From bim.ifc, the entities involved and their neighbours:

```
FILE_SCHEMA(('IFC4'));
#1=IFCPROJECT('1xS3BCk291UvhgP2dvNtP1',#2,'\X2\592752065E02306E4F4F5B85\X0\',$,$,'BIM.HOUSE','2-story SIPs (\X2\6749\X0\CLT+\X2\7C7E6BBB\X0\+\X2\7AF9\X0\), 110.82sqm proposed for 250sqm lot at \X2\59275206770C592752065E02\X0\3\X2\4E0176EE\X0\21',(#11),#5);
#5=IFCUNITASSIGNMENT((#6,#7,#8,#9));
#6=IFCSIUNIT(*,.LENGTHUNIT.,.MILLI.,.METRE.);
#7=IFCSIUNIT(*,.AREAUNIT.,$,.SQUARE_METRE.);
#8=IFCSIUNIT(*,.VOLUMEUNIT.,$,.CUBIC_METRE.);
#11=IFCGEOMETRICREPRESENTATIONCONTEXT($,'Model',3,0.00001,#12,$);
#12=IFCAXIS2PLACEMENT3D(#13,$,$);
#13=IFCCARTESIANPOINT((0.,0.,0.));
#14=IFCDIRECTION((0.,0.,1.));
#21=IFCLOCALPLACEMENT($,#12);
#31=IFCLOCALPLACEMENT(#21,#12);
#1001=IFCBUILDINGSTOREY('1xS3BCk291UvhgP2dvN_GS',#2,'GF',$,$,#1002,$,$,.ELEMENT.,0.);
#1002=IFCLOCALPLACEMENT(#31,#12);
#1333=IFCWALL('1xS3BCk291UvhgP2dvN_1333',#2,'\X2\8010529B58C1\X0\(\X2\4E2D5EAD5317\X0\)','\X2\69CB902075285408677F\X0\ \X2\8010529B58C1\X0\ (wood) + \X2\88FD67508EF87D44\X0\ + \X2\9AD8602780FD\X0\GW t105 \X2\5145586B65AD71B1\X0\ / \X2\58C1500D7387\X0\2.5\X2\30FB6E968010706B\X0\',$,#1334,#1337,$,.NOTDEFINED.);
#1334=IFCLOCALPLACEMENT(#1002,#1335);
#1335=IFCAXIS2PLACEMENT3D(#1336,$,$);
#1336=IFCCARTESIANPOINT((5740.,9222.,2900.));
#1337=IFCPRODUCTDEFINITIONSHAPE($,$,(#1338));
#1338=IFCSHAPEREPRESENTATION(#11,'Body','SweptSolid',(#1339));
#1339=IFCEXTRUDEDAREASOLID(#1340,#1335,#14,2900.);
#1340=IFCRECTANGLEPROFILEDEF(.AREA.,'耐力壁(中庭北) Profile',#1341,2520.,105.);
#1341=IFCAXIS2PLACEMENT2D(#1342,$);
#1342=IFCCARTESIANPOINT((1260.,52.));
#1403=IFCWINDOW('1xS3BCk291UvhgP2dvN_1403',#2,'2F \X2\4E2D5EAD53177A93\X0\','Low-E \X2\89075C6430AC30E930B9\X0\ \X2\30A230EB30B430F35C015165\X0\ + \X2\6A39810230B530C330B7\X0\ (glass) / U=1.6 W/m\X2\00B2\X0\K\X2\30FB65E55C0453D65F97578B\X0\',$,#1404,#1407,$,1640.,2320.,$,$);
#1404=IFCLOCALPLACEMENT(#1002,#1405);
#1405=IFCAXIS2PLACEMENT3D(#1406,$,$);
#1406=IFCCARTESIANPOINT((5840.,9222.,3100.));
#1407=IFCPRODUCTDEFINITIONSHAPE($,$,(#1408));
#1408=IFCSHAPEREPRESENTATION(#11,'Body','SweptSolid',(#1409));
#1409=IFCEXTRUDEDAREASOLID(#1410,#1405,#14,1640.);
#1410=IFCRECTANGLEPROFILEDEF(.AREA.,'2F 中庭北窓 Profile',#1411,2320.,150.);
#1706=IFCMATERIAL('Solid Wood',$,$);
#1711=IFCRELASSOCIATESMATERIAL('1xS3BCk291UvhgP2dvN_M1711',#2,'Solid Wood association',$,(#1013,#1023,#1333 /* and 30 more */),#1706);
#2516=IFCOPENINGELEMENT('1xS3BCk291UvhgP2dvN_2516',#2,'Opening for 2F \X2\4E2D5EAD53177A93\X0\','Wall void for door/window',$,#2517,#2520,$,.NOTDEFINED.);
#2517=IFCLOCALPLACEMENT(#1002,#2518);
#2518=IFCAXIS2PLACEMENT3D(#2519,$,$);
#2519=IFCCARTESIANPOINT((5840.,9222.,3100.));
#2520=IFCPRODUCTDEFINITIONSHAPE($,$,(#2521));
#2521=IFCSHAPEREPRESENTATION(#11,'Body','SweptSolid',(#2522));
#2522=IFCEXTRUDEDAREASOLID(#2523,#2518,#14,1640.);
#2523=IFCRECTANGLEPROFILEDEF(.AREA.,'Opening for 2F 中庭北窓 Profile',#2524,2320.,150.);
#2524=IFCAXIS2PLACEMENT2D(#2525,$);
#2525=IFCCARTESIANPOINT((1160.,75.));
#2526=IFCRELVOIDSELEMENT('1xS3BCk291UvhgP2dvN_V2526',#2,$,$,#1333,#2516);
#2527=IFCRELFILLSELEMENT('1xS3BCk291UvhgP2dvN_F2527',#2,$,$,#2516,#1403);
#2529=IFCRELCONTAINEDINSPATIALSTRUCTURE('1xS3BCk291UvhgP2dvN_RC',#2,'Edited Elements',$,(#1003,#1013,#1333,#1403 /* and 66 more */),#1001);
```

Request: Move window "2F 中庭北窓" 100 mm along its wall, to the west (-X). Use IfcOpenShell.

```python
import ifcopenshell
import ifcopenshell.api.geometry
import ifcopenshell.util.placement
import ifcopenshell.util.unit

model = ifcopenshell.open("bim.ifc")
unit_scale = ifcopenshell.util.unit.calculate_unit_scale(model)

window = model.by_id(1403)
opening = window.FillsVoids[0].RelatingOpeningElement
wall = opening.VoidsElements[0].RelatingBuildingElement

wall_matrix = ifcopenshell.util.placement.get_local_placement(wall.ObjectPlacement)
shift = wall_matrix[:3, 0] * -0.1 / unit_scale
before = ifcopenshell.util.placement.get_local_placement(window.ObjectPlacement)[:3, 3].copy()

# The window is not placed relative to its opening, so move both.
for product in (opening, window):
    matrix = ifcopenshell.util.placement.get_local_placement(product.ObjectPlacement)
    matrix[:3, 3] += shift
    ifcopenshell.api.geometry.edit_object_placement(model, product=product, matrix=matrix, is_si=False)

after = ifcopenshell.util.placement.get_local_placement(window.ObjectPlacement)[:3, 3]
print("window moved by", (after - before).round(3) + 0.0)

model.write("bim-out.ifc")
```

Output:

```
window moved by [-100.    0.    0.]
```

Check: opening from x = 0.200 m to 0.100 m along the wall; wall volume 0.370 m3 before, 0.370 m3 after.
